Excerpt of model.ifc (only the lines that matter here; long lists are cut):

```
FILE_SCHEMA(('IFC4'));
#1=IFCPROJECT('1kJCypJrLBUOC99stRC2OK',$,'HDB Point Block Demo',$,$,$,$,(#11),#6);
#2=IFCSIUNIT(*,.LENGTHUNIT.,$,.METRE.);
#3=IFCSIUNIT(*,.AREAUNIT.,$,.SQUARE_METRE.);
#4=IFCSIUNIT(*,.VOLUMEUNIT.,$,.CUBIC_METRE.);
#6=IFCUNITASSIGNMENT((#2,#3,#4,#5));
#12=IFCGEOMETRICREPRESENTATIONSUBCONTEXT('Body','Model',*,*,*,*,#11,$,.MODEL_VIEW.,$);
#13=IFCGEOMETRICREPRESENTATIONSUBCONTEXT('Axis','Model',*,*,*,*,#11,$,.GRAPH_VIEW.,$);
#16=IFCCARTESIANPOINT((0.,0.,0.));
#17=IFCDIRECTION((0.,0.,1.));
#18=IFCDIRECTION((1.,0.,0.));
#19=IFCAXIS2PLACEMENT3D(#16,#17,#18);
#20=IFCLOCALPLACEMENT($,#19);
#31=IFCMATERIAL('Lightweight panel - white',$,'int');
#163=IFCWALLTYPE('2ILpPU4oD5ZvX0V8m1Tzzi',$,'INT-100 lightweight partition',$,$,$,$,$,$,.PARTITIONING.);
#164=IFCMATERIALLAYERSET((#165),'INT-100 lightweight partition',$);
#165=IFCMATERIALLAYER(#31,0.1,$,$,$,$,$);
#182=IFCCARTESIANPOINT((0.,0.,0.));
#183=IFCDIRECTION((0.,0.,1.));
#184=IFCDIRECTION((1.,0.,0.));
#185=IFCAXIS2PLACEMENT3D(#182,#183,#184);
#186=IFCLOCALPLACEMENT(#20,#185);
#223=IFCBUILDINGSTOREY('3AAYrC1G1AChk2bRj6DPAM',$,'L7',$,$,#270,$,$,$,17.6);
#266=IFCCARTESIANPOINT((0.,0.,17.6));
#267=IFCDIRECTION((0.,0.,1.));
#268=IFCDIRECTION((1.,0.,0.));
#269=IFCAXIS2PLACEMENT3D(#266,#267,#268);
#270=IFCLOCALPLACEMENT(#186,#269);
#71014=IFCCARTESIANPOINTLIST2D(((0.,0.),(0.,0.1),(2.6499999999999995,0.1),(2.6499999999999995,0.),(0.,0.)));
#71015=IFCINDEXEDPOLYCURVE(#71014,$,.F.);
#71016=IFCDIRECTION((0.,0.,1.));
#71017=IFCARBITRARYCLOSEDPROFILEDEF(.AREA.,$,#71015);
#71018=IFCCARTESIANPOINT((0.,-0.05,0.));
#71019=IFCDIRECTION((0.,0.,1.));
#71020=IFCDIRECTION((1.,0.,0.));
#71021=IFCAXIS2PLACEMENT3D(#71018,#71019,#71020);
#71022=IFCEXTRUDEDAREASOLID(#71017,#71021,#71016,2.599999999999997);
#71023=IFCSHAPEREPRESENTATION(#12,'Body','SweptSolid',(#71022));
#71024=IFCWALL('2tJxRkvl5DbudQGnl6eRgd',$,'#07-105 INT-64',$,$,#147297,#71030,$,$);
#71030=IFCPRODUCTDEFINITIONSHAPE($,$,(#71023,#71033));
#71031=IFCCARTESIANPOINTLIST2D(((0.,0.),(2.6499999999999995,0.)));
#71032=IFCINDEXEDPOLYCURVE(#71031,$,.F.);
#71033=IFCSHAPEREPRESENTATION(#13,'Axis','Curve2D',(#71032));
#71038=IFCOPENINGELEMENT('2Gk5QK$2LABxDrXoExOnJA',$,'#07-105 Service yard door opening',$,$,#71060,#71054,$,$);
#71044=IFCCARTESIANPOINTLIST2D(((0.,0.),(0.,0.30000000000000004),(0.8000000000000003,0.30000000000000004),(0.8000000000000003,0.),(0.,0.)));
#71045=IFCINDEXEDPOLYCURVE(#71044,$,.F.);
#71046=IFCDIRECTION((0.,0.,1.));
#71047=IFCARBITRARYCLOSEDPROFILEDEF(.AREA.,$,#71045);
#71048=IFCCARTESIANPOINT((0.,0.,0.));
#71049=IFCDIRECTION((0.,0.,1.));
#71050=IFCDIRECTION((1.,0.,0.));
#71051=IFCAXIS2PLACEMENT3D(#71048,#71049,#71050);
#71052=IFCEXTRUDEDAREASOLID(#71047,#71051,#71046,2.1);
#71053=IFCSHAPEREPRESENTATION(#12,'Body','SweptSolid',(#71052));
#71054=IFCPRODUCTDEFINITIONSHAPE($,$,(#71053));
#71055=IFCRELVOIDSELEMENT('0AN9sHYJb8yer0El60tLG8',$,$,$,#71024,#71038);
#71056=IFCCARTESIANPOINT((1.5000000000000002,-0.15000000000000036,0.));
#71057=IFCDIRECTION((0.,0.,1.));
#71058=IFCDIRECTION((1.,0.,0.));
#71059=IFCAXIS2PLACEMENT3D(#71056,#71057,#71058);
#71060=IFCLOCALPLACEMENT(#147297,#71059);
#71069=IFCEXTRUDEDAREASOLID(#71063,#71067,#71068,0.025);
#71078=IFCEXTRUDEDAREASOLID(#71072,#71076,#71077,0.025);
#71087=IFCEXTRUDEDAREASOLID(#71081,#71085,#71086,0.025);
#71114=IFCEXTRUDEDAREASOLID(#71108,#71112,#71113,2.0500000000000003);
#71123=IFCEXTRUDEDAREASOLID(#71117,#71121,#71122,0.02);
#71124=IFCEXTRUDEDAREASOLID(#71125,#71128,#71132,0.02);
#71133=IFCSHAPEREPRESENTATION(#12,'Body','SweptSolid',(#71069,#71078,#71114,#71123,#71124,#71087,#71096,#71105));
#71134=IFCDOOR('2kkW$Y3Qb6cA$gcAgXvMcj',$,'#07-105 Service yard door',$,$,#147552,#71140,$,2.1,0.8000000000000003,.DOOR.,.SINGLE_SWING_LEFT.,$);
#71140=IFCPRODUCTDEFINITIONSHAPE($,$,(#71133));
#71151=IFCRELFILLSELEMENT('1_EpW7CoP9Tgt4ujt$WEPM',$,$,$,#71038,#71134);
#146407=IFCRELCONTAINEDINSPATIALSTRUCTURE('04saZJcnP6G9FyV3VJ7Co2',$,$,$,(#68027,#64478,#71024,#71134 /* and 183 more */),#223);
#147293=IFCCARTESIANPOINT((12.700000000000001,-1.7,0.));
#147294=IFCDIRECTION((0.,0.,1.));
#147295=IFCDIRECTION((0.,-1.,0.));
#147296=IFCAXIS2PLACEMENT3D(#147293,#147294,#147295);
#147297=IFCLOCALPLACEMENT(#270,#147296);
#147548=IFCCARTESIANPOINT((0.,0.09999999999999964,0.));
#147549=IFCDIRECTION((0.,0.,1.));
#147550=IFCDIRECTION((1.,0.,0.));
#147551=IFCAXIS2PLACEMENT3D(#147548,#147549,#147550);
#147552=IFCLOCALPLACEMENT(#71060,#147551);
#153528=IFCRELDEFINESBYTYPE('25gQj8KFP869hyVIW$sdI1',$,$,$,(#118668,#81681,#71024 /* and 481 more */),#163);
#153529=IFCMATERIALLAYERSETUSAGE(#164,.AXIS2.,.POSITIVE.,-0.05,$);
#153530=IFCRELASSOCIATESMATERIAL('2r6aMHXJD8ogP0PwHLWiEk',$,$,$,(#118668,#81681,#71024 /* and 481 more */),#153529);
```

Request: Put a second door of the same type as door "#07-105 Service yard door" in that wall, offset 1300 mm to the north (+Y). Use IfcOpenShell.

```python
import ifcopenshell
import ifcopenshell.api.feature
import ifcopenshell.api.geometry
import ifcopenshell.api.root
import ifcopenshell.geom
import ifcopenshell.util.element
import ifcopenshell.util.placement
import ifcopenshell.util.shape
import ifcopenshell.util.unit

model = ifcopenshell.open("model.ifc")
unit_scale = ifcopenshell.util.unit.calculate_unit_scale(model)
settings = ifcopenshell.geom.settings()


def volume(element):
    """Net volume in cubic metres, openings subtracted."""
    shape = ifcopenshell.geom.create_shape(settings, element)
    return ifcopenshell.util.shape.get_volume(shape.geometry)


door = model.by_id(71134)
opening = door.FillsVoids[0].RelatingOpeningElement
wall = opening.VoidsElements[0].RelatingBuildingElement
before = volume(wall)
shift = ifcopenshell.util.placement.get_local_placement(wall.ObjectPlacement)[:3, 0] * -1.3 / unit_scale

# copy_class copies the void relationship, type, container and properties, but no geometry.
new_opening = ifcopenshell.api.root.copy_class(model, product=opening)
new_opening.Representation = ifcopenshell.util.element.copy_deep(
    model, opening.Representation, exclude=["IfcGeometricRepresentationContext", "IfcRepresentationMap"]
)
new_door = ifcopenshell.api.root.copy_class(model, product=door)
new_door.Representation = ifcopenshell.util.element.copy_deep(
    model, door.Representation, exclude=["IfcGeometricRepresentationContext", "IfcRepresentationMap"]
)
ifcopenshell.api.feature.add_filling(model, opening=new_opening, element=new_door)

for old, new in ((opening, new_opening), (door, new_door)):
    matrix = ifcopenshell.util.placement.get_local_placement(old.ObjectPlacement)
    matrix[:3, 3] += shift
    ifcopenshell.api.geometry.edit_object_placement(model, product=new, matrix=matrix, is_si=False)

after = volume(wall)

print(f"wall volume {before:.3f} -> {after:.3f} m3")

model.write("model_v2.ifc")
```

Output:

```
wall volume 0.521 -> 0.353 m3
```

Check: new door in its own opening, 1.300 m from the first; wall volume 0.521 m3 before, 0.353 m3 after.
